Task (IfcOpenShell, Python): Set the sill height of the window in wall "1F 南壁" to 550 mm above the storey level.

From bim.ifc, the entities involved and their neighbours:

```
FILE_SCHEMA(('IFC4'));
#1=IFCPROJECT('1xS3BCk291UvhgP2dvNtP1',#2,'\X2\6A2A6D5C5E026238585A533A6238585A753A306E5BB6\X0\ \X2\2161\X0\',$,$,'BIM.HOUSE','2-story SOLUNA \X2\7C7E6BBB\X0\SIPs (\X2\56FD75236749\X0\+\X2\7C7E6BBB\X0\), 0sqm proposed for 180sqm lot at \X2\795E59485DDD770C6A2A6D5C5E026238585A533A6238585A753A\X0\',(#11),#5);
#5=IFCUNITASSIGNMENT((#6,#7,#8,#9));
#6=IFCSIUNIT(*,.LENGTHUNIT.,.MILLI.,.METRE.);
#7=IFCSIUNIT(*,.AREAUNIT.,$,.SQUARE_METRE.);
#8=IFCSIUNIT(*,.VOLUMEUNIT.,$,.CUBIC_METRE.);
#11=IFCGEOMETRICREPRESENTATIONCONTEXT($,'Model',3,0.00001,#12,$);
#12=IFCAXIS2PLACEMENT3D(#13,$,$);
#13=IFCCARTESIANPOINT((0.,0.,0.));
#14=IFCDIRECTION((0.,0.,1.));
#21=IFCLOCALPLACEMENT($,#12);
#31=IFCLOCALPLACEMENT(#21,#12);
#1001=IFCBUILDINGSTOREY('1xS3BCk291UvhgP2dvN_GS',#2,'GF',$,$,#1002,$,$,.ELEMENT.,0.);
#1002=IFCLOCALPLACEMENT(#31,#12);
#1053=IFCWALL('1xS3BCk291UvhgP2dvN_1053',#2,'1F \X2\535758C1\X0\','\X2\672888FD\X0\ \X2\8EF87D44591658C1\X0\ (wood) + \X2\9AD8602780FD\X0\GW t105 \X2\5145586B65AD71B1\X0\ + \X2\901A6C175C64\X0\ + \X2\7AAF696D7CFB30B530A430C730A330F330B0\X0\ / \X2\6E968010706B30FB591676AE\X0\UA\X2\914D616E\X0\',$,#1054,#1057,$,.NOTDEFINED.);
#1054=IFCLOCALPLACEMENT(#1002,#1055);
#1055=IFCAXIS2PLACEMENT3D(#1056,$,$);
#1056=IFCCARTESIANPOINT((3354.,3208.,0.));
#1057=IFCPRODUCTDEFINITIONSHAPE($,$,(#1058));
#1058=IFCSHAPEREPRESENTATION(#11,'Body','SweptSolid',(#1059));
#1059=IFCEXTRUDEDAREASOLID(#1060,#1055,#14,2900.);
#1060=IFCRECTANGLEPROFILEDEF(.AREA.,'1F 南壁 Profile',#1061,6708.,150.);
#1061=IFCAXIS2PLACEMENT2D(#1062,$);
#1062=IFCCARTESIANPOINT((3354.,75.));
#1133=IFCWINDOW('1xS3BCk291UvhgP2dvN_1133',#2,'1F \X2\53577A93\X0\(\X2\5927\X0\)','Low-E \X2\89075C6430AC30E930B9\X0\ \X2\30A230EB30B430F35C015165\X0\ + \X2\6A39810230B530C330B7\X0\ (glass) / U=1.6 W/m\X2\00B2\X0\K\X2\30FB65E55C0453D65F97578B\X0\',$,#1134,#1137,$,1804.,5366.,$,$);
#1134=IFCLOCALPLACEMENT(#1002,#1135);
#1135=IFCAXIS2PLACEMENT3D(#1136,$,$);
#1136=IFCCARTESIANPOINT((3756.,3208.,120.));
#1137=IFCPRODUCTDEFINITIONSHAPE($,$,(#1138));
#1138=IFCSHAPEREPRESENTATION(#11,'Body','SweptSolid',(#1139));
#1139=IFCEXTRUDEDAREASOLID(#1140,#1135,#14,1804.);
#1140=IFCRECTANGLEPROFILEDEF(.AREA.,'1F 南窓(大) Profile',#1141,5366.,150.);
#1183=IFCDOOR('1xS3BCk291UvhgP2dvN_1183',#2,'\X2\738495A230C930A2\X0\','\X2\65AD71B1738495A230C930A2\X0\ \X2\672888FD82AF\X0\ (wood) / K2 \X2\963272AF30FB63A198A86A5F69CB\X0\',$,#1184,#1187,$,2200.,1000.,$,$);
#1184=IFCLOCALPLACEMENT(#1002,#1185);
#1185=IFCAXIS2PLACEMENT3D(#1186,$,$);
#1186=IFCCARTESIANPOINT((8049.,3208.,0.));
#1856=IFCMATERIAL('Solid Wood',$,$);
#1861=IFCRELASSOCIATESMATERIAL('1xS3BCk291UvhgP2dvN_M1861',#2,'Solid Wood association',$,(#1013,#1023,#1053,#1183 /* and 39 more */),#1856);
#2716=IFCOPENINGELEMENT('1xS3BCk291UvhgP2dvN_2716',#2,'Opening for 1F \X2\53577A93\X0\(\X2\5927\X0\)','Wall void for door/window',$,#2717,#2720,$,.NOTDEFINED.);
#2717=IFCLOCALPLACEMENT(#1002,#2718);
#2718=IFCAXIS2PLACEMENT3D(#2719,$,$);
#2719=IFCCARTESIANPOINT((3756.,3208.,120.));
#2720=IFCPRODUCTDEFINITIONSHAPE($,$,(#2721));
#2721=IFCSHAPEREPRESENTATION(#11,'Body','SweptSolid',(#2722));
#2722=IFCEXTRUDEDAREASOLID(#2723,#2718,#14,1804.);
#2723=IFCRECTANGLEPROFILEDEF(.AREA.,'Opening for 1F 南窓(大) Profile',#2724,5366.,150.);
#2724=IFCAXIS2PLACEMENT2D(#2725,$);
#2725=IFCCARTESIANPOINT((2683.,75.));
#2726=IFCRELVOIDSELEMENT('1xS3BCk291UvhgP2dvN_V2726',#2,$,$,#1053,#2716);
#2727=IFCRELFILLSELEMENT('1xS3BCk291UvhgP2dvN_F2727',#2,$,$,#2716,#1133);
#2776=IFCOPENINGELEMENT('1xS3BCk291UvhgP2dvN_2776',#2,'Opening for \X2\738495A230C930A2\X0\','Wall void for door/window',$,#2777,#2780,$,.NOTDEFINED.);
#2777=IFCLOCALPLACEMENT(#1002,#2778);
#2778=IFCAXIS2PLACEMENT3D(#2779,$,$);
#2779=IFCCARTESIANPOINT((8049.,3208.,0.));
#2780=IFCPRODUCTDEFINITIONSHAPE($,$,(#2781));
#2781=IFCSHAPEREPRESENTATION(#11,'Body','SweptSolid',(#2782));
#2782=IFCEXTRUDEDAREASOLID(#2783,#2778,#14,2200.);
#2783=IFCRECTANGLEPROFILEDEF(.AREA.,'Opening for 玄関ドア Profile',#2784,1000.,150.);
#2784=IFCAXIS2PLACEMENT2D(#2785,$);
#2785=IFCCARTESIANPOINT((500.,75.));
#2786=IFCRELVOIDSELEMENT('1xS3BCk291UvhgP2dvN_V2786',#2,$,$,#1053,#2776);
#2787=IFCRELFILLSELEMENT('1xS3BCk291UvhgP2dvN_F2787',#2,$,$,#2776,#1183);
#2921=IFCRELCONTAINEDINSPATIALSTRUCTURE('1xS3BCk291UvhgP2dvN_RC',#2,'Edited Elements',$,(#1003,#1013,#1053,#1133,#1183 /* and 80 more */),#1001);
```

```python
import numpy as np
import ifcopenshell
import ifcopenshell.api.geometry
import ifcopenshell.geom
import ifcopenshell.util.element
import ifcopenshell.util.placement
import ifcopenshell.util.shape
import ifcopenshell.util.unit

model = ifcopenshell.open("bim.ifc")
unit_scale = ifcopenshell.util.unit.calculate_unit_scale(model)

window = model.by_guid("1xS3BCk291UvhgP2dvN_1133")
opening = window.FillsVoids[0].RelatingOpeningElement
storey = ifcopenshell.util.element.get_container(window, ifc_class="IfcBuildingStorey")
level = ifcopenshell.util.placement.get_local_placement(storey.ObjectPlacement)[2, 3]

# The opening's origin need not be at the sill, so measure its lowest point.
shape = ifcopenshell.geom.create_shape(ifcopenshell.geom.settings(), opening)
bottom = ifcopenshell.util.shape.get_shape_bottom_elevation(shape, shape.geometry) / unit_scale
dz = level + 0.55 / unit_scale - bottom

shift = np.array([0.0, 0.0, dz])
# The window is not placed relative to its opening, so move both.
for product in (opening, window):
    matrix = ifcopenshell.util.placement.get_local_placement(product.ObjectPlacement)
    matrix[:3, 3] += shift
    ifcopenshell.api.geometry.edit_object_placement(model, product=product, matrix=matrix, is_si=False)

print(f"moved by {dz * unit_scale:+.3f} m")

model.write("bim_rev.ifc")
```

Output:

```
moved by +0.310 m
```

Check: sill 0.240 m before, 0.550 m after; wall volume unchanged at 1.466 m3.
